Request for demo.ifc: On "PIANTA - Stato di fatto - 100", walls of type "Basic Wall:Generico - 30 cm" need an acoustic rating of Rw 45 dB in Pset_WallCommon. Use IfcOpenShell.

First a look at what the model holds.

```python
import ifcopenshell
import ifcopenshell.util.element

model = ifcopenshell.open("demo.ifc")
print(model.schema)
storey = next(s for s in model.by_type("IfcBuildingStorey") if s.Name == "PIANTA - Stato di fatto - 100")
walls = [e for e in ifcopenshell.util.element.get_decomposition(storey) if e.is_a("IfcWall")]
seen = {}
for e in walls:
    element_type = ifcopenshell.util.element.get_type(e)
    key = (element_type.Name if element_type != e and element_type else None, ifcopenshell.util.element.get_pset(e, "Pset_WallCommon", "AcousticRating"))
    seen[key] = seen.get(key, 0) + 1
for (name, value), count in sorted(seen.items(), key=str):
    print(count, "x", name, "|", value)
```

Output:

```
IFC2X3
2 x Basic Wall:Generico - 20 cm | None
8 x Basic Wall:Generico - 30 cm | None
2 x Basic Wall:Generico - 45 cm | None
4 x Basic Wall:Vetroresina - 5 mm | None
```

```python
import ifcopenshell
import ifcopenshell.api.pset
import ifcopenshell.util.element

model = ifcopenshell.open("demo.ifc")

storey = next(s for s in model.by_type("IfcBuildingStorey") if s.Name == "PIANTA - Stato di fatto - 100")
walls = [e for e in ifcopenshell.util.element.get_decomposition(storey) if e.is_a("IfcWall")]

count = 0
for e in walls:
    element_type = ifcopenshell.util.element.get_type(e)
    if element_type in (None, e) or element_type.Name != "Basic Wall:Generico - 30 cm":
        continue
    # add_pset returns the element's existing set when there is one.
    pset = ifcopenshell.api.pset.add_pset(model, product=e, name="Pset_WallCommon")
    ifcopenshell.api.pset.edit_pset(model, pset=pset, properties={"AcousticRating": "Rw 45 dB"})
    count += 1

print(count, "walls updated")

model.write("demo-out.ifc")
```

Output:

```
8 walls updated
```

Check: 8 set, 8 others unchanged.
